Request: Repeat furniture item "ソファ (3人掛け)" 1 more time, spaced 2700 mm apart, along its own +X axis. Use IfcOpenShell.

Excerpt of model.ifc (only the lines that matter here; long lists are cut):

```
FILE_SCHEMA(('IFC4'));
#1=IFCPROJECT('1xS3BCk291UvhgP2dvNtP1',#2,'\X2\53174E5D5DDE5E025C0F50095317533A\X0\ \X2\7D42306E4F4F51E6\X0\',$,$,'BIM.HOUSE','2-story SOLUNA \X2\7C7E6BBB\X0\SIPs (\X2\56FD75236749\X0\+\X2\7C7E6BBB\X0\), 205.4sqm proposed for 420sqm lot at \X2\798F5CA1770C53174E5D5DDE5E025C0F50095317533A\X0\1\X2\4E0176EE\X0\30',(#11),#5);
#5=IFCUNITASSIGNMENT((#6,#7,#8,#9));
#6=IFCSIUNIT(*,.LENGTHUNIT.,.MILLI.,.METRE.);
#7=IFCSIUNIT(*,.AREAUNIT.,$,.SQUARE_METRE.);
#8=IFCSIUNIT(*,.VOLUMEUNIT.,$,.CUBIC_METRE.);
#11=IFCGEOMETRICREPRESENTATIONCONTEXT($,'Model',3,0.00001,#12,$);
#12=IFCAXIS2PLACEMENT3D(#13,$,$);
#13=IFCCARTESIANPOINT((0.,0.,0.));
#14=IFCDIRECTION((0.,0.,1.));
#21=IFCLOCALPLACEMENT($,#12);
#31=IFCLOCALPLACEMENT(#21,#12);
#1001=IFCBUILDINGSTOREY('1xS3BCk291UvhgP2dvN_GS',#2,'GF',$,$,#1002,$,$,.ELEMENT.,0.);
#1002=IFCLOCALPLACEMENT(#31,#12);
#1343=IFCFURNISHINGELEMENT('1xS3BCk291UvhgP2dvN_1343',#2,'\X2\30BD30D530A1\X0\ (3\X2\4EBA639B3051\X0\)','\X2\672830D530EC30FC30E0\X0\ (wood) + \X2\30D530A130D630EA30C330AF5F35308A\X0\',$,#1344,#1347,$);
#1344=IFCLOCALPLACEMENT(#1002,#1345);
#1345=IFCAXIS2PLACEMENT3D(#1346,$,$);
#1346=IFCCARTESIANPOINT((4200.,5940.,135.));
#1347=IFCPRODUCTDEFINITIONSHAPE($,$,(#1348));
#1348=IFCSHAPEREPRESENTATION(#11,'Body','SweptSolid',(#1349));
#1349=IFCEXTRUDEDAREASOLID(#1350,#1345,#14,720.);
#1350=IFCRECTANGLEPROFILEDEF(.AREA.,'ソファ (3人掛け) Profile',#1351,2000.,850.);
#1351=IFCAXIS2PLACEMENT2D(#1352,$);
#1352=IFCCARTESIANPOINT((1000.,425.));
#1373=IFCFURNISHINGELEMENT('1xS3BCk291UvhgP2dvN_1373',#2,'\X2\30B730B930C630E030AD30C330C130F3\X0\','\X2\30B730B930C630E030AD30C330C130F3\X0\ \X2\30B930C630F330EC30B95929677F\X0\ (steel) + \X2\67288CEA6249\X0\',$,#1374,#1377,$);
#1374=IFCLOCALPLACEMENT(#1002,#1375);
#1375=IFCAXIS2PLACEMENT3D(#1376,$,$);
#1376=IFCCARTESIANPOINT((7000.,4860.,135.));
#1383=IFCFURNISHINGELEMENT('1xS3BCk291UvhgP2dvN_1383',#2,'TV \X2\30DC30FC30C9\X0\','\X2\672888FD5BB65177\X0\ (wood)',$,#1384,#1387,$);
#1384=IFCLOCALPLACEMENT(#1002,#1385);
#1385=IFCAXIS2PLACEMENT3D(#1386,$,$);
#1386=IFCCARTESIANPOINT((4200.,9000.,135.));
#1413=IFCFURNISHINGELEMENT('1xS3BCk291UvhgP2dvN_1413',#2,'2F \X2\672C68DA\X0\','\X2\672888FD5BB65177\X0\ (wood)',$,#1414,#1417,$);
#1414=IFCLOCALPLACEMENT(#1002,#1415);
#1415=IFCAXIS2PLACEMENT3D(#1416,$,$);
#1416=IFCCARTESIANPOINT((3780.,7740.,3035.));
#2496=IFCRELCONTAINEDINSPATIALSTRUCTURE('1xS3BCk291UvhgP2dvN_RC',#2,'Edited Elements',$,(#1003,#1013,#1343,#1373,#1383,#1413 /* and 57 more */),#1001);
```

```python
import ifcopenshell
import ifcopenshell.api.geometry
import ifcopenshell.api.root
import ifcopenshell.util.element
import ifcopenshell.util.placement
import ifcopenshell.util.unit

model = ifcopenshell.open("model.ifc")
unit_scale = ifcopenshell.util.unit.calculate_unit_scale(model)


def reuse_history(source, copy):
    """copy_class also copies each property set's owner history, people and application; keep the originals."""
    for rel in copy.IsDefinedBy:
        if rel.is_a("IfcRelDefinesByProperties") and (history := rel.RelatingPropertyDefinition.OwnerHistory):
            rel.RelatingPropertyDefinition.OwnerHistory = source.OwnerHistory
            ifcopenshell.util.element.remove_deep2(model, history)


source = model.by_guid("1xS3BCk291UvhgP2dvN_1343")
base = ifcopenshell.util.placement.get_local_placement(source.ObjectPlacement)
step = base[:3, 0] * 2.7 / unit_scale

for i in range(1, 2):
    copy = ifcopenshell.api.root.copy_class(model, product=source)
    copy.Representation = ifcopenshell.util.element.copy_deep(
        model, source.Representation, exclude=["IfcGeometricRepresentationContext", "IfcRepresentationMap"]
    )
    reuse_history(source, copy)
    matrix = base.copy()
    matrix[:3, 3] += i * step
    print("added at", matrix[:3, 3].round(3) + 0.0)
    ifcopenshell.api.geometry.edit_object_placement(model, product=copy, matrix=matrix, is_si=False)

model.write("model-out.ifc")
```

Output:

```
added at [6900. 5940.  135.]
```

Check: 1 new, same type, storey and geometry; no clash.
